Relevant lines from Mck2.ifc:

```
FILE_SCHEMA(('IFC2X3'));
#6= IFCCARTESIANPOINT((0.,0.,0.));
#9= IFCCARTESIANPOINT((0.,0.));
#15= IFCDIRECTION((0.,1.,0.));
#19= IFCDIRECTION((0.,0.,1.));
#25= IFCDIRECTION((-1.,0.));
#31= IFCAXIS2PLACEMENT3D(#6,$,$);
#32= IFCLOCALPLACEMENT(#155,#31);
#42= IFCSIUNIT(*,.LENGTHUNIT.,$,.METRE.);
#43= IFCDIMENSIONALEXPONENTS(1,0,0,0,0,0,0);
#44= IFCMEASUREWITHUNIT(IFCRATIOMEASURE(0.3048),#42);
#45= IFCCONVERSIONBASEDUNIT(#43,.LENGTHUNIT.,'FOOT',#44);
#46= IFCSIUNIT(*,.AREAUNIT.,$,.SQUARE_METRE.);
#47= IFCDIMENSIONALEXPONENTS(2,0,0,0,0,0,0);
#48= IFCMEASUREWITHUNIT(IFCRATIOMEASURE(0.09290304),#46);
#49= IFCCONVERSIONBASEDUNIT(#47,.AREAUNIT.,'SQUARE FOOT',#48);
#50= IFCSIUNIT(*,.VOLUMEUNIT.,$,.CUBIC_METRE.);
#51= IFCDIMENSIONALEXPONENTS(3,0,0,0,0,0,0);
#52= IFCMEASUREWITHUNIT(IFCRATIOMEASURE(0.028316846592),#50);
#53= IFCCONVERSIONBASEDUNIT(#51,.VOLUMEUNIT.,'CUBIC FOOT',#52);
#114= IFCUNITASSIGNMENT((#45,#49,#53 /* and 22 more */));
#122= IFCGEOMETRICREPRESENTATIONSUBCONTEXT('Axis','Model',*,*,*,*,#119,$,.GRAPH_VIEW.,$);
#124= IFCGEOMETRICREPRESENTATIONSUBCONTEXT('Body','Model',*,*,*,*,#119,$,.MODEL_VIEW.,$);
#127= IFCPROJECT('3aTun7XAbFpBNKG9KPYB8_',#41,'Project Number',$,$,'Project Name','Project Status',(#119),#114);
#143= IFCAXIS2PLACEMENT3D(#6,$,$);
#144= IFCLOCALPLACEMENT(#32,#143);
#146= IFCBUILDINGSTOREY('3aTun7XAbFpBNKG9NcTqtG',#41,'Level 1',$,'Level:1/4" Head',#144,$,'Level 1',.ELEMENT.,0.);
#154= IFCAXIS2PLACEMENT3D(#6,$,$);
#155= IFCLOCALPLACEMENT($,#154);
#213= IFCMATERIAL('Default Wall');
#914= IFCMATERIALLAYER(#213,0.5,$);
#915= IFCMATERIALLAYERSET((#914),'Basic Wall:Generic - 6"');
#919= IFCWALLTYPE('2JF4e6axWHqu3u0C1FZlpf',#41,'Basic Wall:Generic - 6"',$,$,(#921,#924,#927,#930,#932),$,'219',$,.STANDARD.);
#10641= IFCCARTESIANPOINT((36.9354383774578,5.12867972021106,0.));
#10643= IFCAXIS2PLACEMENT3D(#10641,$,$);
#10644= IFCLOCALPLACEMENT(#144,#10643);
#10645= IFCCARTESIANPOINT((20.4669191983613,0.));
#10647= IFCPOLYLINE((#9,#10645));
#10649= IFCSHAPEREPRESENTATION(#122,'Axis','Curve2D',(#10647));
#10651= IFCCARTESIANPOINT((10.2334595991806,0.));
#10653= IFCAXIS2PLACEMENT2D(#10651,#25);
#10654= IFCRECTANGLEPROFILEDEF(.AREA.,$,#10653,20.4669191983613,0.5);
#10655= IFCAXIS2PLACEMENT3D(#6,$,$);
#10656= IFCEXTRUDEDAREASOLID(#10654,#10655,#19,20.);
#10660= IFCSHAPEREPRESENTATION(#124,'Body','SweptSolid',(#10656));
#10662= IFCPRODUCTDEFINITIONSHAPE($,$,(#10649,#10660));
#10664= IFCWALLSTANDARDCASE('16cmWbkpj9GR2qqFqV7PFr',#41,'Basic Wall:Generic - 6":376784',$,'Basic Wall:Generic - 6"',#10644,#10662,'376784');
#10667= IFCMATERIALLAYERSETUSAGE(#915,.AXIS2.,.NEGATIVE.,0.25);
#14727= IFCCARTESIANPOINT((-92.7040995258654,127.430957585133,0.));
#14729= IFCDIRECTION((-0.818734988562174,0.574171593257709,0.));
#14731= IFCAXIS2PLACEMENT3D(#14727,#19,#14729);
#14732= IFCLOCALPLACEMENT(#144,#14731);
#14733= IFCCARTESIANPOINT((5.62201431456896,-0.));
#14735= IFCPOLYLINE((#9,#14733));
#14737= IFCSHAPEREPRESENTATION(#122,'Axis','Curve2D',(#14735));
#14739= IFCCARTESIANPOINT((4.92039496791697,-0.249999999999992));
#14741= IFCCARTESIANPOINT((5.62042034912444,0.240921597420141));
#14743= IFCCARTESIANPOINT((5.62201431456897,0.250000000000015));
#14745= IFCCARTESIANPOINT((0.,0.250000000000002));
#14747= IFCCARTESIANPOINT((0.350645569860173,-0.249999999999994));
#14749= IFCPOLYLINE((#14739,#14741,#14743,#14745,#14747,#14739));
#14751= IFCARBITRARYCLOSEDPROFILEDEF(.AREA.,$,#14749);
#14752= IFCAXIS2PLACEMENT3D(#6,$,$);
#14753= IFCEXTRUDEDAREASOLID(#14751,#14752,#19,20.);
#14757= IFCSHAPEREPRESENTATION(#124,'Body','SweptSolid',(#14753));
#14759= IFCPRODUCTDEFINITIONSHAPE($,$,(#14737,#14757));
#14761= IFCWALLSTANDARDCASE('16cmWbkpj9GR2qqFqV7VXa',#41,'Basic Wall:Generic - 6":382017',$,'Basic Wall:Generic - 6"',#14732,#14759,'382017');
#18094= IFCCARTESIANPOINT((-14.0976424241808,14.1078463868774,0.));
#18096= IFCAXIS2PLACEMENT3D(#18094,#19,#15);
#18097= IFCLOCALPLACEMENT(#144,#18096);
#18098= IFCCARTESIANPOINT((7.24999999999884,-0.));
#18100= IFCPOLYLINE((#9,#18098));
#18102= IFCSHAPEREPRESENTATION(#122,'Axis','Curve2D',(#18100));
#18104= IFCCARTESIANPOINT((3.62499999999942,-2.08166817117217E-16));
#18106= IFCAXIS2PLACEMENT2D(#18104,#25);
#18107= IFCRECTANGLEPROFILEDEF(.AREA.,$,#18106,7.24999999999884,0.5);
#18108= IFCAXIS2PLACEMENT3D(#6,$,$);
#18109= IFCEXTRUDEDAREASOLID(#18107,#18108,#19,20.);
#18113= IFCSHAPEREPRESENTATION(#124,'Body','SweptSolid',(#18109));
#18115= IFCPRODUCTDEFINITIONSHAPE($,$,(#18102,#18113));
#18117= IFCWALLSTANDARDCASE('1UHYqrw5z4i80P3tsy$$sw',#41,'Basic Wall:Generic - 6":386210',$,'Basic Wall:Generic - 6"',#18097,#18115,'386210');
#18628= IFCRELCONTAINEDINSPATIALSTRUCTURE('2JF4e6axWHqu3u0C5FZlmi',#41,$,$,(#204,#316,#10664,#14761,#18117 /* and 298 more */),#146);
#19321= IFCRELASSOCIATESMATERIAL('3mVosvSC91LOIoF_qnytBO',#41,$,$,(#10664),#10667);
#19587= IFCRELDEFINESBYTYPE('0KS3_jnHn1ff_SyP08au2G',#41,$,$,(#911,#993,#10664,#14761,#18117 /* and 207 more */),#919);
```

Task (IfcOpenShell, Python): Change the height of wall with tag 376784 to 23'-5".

```python
import ifcopenshell
import ifcopenshell.geom
import ifcopenshell.util.representation
import ifcopenshell.util.shape
import ifcopenshell.util.unit

model = ifcopenshell.open("Mck2.ifc")
unit_scale = ifcopenshell.util.unit.calculate_unit_scale(model)
settings = ifcopenshell.geom.settings()


def volume(element):
    """Net volume in cubic metres, openings subtracted."""
    shape = ifcopenshell.geom.create_shape(settings, element)
    return ifcopenshell.util.shape.get_volume(shape.geometry)


wall = model.by_id(10664)
before = volume(wall)

body = ifcopenshell.util.representation.get_representation(wall, "Model", "Body")
solid = body.Items[0]
old_height = solid.Depth
solid.Depth = 281 * 0.0254 / unit_scale
after = volume(wall)

print(f"height {old_height:g} -> {solid.Depth:g}, volume {before:.3f} -> {after:.3f} m3")

model.write("Mck2_edited.ifc")
```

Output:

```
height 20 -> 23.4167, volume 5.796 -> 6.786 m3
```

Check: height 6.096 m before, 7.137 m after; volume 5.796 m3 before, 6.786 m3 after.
